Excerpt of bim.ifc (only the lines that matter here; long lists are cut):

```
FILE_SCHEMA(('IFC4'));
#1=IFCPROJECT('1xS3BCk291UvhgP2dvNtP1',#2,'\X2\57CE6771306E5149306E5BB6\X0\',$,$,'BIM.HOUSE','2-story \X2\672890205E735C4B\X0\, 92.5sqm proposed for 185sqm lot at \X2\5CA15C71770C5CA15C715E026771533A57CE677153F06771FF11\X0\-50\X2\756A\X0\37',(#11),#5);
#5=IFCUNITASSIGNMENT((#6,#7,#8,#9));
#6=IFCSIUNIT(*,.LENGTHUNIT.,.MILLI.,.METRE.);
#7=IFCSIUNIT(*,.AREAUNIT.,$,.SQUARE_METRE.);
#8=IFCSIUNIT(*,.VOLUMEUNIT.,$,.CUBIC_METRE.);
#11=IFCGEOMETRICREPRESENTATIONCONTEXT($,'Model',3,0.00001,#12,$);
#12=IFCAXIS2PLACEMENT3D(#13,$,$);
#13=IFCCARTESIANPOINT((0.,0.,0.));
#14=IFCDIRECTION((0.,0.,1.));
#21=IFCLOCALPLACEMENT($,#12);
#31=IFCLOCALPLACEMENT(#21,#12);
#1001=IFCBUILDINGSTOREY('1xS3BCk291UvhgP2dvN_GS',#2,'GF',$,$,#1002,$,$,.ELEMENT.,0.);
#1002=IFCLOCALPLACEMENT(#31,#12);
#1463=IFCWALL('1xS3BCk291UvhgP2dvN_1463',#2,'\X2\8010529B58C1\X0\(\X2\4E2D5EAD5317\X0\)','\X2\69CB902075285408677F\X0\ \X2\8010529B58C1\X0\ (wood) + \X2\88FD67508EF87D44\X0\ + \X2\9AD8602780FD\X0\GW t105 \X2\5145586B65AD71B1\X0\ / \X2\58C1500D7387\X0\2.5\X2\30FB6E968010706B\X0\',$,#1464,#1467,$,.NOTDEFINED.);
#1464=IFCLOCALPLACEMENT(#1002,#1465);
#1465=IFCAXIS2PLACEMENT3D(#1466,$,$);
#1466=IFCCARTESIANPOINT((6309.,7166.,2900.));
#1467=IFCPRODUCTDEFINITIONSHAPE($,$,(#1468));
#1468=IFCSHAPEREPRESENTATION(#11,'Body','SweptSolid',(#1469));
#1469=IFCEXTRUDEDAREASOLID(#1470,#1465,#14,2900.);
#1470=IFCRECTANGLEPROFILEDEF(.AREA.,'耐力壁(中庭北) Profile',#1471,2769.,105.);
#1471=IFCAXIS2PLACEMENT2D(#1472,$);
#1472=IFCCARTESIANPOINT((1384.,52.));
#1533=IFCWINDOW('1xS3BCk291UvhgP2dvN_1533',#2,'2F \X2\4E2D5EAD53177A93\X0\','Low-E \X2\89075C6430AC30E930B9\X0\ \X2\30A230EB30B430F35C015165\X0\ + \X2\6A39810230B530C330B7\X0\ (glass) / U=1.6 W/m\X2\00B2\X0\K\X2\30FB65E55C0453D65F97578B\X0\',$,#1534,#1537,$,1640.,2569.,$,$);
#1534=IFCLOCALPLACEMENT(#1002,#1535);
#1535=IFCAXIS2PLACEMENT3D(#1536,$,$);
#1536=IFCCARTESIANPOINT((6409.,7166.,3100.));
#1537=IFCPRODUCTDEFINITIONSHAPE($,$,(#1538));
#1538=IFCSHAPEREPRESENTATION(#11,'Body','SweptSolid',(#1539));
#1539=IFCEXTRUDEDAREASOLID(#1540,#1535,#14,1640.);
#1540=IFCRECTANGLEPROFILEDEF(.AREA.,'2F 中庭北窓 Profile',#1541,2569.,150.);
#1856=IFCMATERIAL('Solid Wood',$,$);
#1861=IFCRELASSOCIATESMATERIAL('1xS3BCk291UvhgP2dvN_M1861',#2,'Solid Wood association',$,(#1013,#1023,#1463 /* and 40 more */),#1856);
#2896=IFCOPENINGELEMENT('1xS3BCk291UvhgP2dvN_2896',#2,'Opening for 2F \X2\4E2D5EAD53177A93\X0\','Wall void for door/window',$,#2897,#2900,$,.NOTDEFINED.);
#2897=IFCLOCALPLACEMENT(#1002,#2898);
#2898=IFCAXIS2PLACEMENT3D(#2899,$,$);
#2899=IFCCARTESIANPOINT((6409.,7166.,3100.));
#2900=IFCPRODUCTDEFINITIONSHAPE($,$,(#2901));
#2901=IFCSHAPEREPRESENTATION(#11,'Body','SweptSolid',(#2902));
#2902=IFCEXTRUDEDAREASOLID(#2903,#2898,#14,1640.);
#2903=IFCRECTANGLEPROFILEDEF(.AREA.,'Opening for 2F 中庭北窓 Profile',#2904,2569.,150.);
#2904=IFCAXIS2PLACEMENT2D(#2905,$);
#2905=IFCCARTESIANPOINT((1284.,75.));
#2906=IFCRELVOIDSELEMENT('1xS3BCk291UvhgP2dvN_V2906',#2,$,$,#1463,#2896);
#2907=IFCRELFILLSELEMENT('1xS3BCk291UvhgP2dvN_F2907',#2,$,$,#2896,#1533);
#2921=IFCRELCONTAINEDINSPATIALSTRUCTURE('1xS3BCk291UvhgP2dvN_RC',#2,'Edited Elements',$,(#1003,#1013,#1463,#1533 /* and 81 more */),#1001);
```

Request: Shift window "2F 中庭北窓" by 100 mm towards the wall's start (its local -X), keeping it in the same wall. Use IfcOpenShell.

```python
import ifcopenshell
import ifcopenshell.api.geometry
import ifcopenshell.util.placement
import ifcopenshell.util.unit

model = ifcopenshell.open("bim.ifc")
unit_scale = ifcopenshell.util.unit.calculate_unit_scale(model)

window = model.by_guid("1xS3BCk291UvhgP2dvN_1533")
opening = window.FillsVoids[0].RelatingOpeningElement
wall = opening.VoidsElements[0].RelatingBuildingElement

wall_matrix = ifcopenshell.util.placement.get_local_placement(wall.ObjectPlacement)
shift = wall_matrix[:3, 0] * -0.1 / unit_scale
before = ifcopenshell.util.placement.get_local_placement(window.ObjectPlacement)[:3, 3].copy()

# The window is not placed relative to its opening, so move both.
for product in (opening, window):
    matrix = ifcopenshell.util.placement.get_local_placement(product.ObjectPlacement)
    matrix[:3, 3] += shift
    ifcopenshell.api.geometry.edit_object_placement(model, product=product, matrix=matrix, is_si=False)

after = ifcopenshell.util.placement.get_local_placement(window.ObjectPlacement)[:3, 3]
print("window moved by", (after - before).round(3) + 0.0)

model.write("bim_rev.ifc")
```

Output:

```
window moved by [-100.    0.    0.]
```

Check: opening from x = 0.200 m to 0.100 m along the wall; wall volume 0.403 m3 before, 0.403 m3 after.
